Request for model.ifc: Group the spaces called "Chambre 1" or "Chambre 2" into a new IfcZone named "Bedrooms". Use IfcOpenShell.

First a look at what the model holds.

```python
import ifcopenshell

model = ifcopenshell.open("model.ifc")
print(model.schema)
seen = {}
for space in model.by_type("IfcSpace"):
    seen[space.LongName] = seen.get(space.LongName, 0) + 1
for name, count in sorted(seen.items(), key=str):
    print(count, "x", name)
print("zones:", [z.Name for z in model.by_type("IfcZone")][:20])
```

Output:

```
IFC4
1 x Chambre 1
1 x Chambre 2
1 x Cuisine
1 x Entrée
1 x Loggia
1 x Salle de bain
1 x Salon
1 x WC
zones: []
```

```python
import ifcopenshell
import ifcopenshell.api.group
import ifcopenshell.api.root

model = ifcopenshell.open("model.ifc")

names = {"Chambre 1", "Chambre 2"}
spaces = [s for s in model.by_type("IfcSpace") if s.LongName in names]

zone = ifcopenshell.api.root.create_entity(model, ifc_class="IfcZone", name="Bedrooms")
ifcopenshell.api.group.assign_group(model, products=spaces, group=zone)
print(len(spaces), "spaces in", zone.Name)

model.write("model_v2.ifc")
```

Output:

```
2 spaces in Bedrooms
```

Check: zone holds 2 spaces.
